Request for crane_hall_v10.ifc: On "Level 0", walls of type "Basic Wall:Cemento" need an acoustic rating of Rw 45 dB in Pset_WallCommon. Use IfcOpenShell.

First a look at what the model holds.

```python
import ifcopenshell
import ifcopenshell.util.element

model = ifcopenshell.open("crane_hall_v10.ifc")
print(model.schema)
storey = next(s for s in model.by_type("IfcBuildingStorey") if s.Name == "Level 0")
walls = [e for e in ifcopenshell.util.element.get_decomposition(storey) if e.is_a("IfcWall")]
seen = {}
for e in walls:
    element_type = ifcopenshell.util.element.get_type(e)
    key = (element_type.Name if element_type != e and element_type else None, ifcopenshell.util.element.get_pset(e, "Pset_WallCommon", "AcousticRating"))
    seen[key] = seen.get(key, 0) + 1
for (name, value), count in sorted(seen.items(), key=str):
    print(count, "x", name, "|", value)
```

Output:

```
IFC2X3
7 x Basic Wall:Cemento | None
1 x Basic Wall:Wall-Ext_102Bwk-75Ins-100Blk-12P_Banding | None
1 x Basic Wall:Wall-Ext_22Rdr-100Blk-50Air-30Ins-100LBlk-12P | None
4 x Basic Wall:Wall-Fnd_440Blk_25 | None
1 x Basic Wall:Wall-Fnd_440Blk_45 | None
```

```python
import ifcopenshell
import ifcopenshell.api.pset
import ifcopenshell.util.element

model = ifcopenshell.open("crane_hall_v10.ifc")

storey = next(s for s in model.by_type("IfcBuildingStorey") if s.Name == "Level 0")
walls = [e for e in ifcopenshell.util.element.get_decomposition(storey) if e.is_a("IfcWall")]

count = 0
for e in walls:
    element_type = ifcopenshell.util.element.get_type(e)
    if element_type in (None, e) or element_type.Name != "Basic Wall:Cemento":
        continue
    # add_pset returns the element's existing set when there is one.
    pset = ifcopenshell.api.pset.add_pset(model, product=e, name="Pset_WallCommon")
    ifcopenshell.api.pset.edit_pset(model, pset=pset, properties={"AcousticRating": "Rw 45 dB"})
    count += 1

print(count, "walls updated")

model.write("crane_hall_v10_rev.ifc")
```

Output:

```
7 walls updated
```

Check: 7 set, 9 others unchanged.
